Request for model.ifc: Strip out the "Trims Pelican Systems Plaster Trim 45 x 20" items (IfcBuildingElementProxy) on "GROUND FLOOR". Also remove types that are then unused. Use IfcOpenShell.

First a look at what the model holds.

```python
import ifcopenshell
import ifcopenshell.util.element

model = ifcopenshell.open("model.ifc")
print(model.schema)
storey = next(s for s in model.by_type("IfcBuildingStorey") if s.Name == "GROUND FLOOR")
proxies = [e for e in ifcopenshell.util.element.get_decomposition(storey) if e.is_a("IfcBuildingElementProxy")]
seen = {}
for e in proxies:
    element_type = ifcopenshell.util.element.get_type(e)
    name = element_type.Name if element_type not in (None, e) else None
    seen[name] = seen.get(name, 0) + 1
for name, count in sorted(seen.items(), key=str):
    print(count, "x", name)
```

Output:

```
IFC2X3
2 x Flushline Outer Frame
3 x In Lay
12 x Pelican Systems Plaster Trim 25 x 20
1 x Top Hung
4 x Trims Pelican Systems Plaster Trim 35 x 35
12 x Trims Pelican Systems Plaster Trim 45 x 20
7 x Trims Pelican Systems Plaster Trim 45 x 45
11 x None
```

```python
import ifcopenshell
import ifcopenshell.api.root
import ifcopenshell.util.element

model = ifcopenshell.open("model.ifc")

storey = next(s for s in model.by_type("IfcBuildingStorey") if s.Name == "GROUND FLOOR")
proxies = [e for e in ifcopenshell.util.element.get_decomposition(storey) if e.is_a("IfcBuildingElementProxy")]
targets = [e for e in proxies if (t := ifcopenshell.util.element.get_type(e)) not in (None, e) and t.Name == "Trims Pelican Systems Plaster Trim 45 x 20"]
types = {ifcopenshell.util.element.get_type(e) for e in targets} - {None, *targets}

for e in targets:
    ifcopenshell.api.root.remove_product(model, product=e)
print(len(targets), "removed")

unused = [t for t in types if not ifcopenshell.util.element.get_types(t)]
for t in unused:
    ifcopenshell.api.root.remove_product(model, product=t)
print(len(unused), "unused types removed")

model.write("model_v2.ifc")
```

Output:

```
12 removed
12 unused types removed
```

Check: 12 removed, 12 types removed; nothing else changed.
